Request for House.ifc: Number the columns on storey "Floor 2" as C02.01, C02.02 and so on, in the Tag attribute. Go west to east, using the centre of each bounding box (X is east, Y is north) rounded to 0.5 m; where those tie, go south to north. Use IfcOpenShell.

First a look at what the model holds.

```python
import ifcopenshell
import ifcopenshell.util.element
import ifcopenshell.util.placement

model = ifcopenshell.open("House.ifc")
print(model.schema)
storey = next(s for s in model.by_type("IfcBuildingStorey") if s.Name == "Floor 2")
columns = [e for e in ifcopenshell.util.element.get_decomposition(storey) if e.is_a("IfcColumn")]
for e in sorted(columns, key=lambda e: e.id()):
    origin = ifcopenshell.util.placement.get_local_placement(e.ObjectPlacement)[:3, 3]
    print(e.id(), e.Tag, e.Name, origin.round(2) + 0.0, sep=" | ")
```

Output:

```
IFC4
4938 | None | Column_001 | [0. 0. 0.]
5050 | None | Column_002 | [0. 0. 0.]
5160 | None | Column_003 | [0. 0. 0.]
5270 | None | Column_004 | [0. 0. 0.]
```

```python
import ifcopenshell
import ifcopenshell.geom
import ifcopenshell.util.element
import ifcopenshell.util.shape

model = ifcopenshell.open("House.ifc")
settings = ifcopenshell.geom.settings()
settings.set("use-world-coords", True)


def centre(element):
    shape = ifcopenshell.geom.create_shape(settings, element)
    return ifcopenshell.util.shape.get_bbox_centroid(shape.geometry)


storey = next(s for s in model.by_type("IfcBuildingStorey") if s.Name == "Floor 2")
columns = [e for e in ifcopenshell.util.element.get_decomposition(storey) if e.is_a("IfcColumn")]

# Insertion points can sit at a corner or the storey origin, so sort by the geometry (in metres).
centres = {e: centre(e) for e in columns}
columns.sort(key=lambda e: (round(centres[e][0] / 0.5), centres[e][1]))

for i, e in enumerate(columns, start=1):
    number = f"C02.{i:02d}"
    e.Tag = number
    print(e.id(), number)

model.write("House_rev.ifc")
```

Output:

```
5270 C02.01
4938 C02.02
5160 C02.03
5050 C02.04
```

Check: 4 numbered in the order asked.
